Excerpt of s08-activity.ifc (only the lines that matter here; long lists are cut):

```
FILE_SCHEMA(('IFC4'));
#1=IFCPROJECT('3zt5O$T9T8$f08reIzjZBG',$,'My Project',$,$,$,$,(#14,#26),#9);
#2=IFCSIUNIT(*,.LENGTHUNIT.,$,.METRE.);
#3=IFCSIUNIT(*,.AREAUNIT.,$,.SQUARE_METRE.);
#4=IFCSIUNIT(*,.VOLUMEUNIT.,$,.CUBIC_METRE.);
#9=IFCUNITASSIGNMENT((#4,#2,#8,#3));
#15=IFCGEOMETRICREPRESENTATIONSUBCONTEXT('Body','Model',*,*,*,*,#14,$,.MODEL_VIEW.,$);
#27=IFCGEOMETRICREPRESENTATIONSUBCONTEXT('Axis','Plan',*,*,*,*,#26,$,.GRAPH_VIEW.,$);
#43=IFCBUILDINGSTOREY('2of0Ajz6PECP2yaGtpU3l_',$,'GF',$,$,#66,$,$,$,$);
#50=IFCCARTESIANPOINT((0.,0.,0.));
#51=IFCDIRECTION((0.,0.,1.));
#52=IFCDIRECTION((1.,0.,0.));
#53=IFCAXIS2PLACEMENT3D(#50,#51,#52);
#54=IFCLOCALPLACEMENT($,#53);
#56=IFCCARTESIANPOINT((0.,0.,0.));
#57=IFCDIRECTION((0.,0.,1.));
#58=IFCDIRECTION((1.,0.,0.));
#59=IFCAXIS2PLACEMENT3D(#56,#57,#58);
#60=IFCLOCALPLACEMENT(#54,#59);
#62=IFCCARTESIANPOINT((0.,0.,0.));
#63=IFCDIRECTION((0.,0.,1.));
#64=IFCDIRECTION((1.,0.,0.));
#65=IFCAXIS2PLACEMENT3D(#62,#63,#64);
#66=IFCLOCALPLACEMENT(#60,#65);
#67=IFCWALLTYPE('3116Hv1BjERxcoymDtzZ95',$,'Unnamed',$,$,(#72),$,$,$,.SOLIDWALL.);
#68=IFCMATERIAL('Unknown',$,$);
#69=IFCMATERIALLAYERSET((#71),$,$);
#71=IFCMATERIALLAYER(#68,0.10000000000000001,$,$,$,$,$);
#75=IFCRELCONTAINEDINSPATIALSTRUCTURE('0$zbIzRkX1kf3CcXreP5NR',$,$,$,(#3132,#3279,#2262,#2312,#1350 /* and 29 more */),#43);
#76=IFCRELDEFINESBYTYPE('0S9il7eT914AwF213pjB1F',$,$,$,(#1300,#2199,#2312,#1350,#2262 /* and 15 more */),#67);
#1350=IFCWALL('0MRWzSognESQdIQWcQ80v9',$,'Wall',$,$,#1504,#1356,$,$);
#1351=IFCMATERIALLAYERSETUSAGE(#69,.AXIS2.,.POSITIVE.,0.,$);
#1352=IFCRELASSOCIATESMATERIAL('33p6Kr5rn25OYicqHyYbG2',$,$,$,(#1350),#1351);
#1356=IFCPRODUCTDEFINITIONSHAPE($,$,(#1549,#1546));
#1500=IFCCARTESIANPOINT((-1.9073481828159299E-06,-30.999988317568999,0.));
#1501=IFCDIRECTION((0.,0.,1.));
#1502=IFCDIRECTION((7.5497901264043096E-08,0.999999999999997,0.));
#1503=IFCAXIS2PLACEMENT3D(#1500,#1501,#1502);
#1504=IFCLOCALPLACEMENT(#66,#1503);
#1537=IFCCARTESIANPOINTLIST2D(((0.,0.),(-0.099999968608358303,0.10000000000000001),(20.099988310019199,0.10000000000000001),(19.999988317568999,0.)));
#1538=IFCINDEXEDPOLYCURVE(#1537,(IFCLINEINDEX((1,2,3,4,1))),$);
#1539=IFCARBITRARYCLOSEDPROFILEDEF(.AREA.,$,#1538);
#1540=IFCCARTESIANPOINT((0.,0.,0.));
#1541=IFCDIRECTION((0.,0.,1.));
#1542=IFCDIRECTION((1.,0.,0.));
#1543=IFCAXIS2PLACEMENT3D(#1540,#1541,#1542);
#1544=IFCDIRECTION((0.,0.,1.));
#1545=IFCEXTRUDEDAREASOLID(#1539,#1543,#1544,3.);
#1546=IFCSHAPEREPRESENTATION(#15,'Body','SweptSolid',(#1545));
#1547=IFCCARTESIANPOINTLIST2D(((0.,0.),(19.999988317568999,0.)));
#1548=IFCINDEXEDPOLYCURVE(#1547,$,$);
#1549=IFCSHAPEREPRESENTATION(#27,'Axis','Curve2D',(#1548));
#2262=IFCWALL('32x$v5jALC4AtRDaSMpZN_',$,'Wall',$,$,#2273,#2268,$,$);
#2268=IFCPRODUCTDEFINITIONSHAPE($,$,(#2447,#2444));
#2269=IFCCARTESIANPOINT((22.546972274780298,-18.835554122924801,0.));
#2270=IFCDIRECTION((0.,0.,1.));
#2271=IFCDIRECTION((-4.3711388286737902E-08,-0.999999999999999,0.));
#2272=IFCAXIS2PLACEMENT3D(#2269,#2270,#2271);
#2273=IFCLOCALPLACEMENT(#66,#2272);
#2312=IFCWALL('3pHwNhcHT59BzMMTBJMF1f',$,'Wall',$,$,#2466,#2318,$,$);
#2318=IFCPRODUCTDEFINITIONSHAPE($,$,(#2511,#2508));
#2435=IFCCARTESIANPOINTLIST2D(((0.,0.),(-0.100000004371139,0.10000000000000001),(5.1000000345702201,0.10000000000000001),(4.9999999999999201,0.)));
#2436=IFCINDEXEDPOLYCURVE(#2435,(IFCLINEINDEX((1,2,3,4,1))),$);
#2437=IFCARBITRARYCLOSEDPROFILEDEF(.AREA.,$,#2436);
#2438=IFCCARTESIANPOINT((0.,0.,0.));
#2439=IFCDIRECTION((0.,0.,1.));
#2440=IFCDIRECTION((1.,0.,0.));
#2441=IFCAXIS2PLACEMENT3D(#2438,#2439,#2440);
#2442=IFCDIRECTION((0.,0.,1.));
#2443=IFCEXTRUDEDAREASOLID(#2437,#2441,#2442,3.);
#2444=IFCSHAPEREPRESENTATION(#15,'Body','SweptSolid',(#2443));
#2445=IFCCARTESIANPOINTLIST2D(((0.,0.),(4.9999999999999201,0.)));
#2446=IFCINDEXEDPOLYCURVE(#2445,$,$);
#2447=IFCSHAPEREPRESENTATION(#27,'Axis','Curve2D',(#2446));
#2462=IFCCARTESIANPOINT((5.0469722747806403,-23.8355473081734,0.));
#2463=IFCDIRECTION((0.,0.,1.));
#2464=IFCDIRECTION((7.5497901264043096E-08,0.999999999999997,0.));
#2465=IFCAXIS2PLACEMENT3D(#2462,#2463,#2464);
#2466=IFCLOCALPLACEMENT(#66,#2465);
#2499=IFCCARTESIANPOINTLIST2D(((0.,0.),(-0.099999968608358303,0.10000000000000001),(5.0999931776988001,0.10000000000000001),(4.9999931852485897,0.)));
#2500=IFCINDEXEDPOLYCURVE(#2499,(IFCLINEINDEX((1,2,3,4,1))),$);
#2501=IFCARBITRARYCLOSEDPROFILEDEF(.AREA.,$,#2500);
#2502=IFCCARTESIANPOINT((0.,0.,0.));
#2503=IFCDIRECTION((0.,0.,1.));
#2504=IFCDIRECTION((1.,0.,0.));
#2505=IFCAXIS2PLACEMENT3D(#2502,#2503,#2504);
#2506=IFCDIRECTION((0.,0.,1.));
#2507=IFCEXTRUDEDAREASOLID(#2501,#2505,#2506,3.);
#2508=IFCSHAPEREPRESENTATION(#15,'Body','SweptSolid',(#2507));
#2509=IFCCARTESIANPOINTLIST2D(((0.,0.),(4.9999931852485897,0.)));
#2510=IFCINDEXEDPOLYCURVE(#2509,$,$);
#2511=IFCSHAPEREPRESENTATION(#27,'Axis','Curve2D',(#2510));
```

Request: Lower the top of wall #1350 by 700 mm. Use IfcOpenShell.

```python
import ifcopenshell
import ifcopenshell.geom
import ifcopenshell.util.representation
import ifcopenshell.util.shape
import ifcopenshell.util.unit

model = ifcopenshell.open("s08-activity.ifc")
unit_scale = ifcopenshell.util.unit.calculate_unit_scale(model)
settings = ifcopenshell.geom.settings()


def volume(element):
    """Net volume in cubic metres, openings subtracted."""
    shape = ifcopenshell.geom.create_shape(settings, element)
    return ifcopenshell.util.shape.get_volume(shape.geometry)


wall = model.by_guid("0MRWzSognESQdIQWcQ80v9")
before = volume(wall)

body = ifcopenshell.util.representation.get_representation(wall, "Model", "Body")
solid = body.Items[0]
old_height = solid.Depth
solid.Depth -= 0.7 / unit_scale
after = volume(wall)

print(f"height {old_height:g} -> {solid.Depth:g}, volume {before:.3f} -> {after:.3f} m3")

model.write("s08-activity_rev.ifc")
```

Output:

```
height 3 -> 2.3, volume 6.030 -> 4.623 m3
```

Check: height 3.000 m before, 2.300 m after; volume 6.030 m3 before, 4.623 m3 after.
